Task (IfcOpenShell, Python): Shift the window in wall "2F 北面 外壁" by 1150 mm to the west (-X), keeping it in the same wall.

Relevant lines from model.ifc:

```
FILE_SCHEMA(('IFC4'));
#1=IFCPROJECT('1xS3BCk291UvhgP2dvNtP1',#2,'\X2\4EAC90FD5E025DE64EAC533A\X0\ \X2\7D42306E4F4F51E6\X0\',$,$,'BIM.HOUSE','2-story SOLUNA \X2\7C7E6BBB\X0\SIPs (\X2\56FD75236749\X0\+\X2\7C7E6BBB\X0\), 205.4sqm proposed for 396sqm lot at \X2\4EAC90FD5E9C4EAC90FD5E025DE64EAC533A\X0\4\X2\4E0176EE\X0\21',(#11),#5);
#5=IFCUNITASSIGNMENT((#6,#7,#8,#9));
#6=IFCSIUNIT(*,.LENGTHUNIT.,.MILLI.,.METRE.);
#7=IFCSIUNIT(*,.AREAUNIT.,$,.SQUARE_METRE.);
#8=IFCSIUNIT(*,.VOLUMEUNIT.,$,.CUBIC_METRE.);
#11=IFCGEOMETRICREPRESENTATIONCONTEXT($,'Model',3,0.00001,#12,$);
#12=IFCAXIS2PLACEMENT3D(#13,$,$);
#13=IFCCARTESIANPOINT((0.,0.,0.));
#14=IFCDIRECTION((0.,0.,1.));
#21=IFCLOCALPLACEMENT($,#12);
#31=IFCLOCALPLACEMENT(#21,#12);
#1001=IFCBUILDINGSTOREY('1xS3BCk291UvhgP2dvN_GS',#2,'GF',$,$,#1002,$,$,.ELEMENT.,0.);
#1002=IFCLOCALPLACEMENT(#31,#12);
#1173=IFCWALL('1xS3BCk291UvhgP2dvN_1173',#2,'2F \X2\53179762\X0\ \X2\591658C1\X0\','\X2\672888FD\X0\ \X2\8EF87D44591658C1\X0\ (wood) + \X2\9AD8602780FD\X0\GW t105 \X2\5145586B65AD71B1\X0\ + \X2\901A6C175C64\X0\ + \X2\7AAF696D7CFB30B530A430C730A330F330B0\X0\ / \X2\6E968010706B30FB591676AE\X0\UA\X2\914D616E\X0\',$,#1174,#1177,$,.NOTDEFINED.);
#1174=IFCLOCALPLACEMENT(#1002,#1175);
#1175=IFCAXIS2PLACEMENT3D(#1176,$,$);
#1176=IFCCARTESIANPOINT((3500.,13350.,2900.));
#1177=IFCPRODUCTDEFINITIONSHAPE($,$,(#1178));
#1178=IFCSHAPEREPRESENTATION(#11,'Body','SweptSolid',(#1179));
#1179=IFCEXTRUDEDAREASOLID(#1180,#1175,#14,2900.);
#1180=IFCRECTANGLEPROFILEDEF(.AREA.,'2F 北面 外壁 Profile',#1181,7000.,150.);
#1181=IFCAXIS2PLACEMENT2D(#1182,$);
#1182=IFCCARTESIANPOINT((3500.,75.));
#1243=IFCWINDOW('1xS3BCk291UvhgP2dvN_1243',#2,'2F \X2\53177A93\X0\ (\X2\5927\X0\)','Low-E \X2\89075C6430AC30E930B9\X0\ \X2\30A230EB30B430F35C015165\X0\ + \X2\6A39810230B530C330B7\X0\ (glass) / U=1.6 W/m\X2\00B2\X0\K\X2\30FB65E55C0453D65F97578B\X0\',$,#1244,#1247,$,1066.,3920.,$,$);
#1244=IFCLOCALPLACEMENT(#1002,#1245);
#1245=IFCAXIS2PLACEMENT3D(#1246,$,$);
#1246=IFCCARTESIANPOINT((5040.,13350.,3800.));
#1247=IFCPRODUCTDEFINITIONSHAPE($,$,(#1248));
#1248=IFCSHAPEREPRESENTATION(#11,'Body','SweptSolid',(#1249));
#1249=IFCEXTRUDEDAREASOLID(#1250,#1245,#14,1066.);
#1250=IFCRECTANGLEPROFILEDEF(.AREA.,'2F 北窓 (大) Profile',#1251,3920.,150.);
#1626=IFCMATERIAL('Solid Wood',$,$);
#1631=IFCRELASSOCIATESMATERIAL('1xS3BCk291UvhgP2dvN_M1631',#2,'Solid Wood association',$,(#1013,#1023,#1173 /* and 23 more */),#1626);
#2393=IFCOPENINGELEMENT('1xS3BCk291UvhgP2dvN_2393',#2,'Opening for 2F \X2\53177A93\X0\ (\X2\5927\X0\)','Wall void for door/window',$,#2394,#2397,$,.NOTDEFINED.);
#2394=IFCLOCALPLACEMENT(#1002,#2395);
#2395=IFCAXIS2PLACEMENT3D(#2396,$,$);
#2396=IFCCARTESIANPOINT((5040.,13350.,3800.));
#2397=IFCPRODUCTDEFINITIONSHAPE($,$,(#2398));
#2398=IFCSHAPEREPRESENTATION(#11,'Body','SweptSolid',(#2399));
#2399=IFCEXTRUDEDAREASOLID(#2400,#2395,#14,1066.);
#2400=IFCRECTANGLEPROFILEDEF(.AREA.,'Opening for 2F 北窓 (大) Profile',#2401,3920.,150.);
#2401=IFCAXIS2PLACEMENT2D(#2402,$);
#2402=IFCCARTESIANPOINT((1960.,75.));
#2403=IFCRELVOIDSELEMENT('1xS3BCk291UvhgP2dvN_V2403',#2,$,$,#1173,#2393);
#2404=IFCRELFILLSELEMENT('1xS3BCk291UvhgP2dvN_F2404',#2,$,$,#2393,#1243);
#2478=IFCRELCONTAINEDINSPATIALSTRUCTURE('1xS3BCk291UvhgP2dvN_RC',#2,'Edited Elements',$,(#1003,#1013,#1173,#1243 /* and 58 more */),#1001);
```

```python
import ifcopenshell
import ifcopenshell.api.geometry
import ifcopenshell.util.placement

model = ifcopenshell.open("model.ifc")

window = model.by_guid("1xS3BCk291UvhgP2dvN_1243")
opening = window.FillsVoids[0].RelatingOpeningElement
wall = opening.VoidsElements[0].RelatingBuildingElement

wall_matrix = ifcopenshell.util.placement.get_local_placement(wall.ObjectPlacement)
shift = wall_matrix[:3, 0] * -1150.0
before = ifcopenshell.util.placement.get_local_placement(window.ObjectPlacement)[:3, 3].copy()

# The window is not placed relative to its opening, so move both.
for product in (opening, window):
    matrix = ifcopenshell.util.placement.get_local_placement(product.ObjectPlacement)
    matrix[:3, 3] += shift
    ifcopenshell.api.geometry.edit_object_placement(model, product=product, matrix=matrix, is_si=False)

after = ifcopenshell.util.placement.get_local_placement(window.ObjectPlacement)[:3, 3]
print("window moved by", (after - before).round(3) + 0.0)

model.write("model_edited.ifc")
```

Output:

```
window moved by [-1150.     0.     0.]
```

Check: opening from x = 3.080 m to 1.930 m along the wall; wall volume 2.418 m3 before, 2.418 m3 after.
